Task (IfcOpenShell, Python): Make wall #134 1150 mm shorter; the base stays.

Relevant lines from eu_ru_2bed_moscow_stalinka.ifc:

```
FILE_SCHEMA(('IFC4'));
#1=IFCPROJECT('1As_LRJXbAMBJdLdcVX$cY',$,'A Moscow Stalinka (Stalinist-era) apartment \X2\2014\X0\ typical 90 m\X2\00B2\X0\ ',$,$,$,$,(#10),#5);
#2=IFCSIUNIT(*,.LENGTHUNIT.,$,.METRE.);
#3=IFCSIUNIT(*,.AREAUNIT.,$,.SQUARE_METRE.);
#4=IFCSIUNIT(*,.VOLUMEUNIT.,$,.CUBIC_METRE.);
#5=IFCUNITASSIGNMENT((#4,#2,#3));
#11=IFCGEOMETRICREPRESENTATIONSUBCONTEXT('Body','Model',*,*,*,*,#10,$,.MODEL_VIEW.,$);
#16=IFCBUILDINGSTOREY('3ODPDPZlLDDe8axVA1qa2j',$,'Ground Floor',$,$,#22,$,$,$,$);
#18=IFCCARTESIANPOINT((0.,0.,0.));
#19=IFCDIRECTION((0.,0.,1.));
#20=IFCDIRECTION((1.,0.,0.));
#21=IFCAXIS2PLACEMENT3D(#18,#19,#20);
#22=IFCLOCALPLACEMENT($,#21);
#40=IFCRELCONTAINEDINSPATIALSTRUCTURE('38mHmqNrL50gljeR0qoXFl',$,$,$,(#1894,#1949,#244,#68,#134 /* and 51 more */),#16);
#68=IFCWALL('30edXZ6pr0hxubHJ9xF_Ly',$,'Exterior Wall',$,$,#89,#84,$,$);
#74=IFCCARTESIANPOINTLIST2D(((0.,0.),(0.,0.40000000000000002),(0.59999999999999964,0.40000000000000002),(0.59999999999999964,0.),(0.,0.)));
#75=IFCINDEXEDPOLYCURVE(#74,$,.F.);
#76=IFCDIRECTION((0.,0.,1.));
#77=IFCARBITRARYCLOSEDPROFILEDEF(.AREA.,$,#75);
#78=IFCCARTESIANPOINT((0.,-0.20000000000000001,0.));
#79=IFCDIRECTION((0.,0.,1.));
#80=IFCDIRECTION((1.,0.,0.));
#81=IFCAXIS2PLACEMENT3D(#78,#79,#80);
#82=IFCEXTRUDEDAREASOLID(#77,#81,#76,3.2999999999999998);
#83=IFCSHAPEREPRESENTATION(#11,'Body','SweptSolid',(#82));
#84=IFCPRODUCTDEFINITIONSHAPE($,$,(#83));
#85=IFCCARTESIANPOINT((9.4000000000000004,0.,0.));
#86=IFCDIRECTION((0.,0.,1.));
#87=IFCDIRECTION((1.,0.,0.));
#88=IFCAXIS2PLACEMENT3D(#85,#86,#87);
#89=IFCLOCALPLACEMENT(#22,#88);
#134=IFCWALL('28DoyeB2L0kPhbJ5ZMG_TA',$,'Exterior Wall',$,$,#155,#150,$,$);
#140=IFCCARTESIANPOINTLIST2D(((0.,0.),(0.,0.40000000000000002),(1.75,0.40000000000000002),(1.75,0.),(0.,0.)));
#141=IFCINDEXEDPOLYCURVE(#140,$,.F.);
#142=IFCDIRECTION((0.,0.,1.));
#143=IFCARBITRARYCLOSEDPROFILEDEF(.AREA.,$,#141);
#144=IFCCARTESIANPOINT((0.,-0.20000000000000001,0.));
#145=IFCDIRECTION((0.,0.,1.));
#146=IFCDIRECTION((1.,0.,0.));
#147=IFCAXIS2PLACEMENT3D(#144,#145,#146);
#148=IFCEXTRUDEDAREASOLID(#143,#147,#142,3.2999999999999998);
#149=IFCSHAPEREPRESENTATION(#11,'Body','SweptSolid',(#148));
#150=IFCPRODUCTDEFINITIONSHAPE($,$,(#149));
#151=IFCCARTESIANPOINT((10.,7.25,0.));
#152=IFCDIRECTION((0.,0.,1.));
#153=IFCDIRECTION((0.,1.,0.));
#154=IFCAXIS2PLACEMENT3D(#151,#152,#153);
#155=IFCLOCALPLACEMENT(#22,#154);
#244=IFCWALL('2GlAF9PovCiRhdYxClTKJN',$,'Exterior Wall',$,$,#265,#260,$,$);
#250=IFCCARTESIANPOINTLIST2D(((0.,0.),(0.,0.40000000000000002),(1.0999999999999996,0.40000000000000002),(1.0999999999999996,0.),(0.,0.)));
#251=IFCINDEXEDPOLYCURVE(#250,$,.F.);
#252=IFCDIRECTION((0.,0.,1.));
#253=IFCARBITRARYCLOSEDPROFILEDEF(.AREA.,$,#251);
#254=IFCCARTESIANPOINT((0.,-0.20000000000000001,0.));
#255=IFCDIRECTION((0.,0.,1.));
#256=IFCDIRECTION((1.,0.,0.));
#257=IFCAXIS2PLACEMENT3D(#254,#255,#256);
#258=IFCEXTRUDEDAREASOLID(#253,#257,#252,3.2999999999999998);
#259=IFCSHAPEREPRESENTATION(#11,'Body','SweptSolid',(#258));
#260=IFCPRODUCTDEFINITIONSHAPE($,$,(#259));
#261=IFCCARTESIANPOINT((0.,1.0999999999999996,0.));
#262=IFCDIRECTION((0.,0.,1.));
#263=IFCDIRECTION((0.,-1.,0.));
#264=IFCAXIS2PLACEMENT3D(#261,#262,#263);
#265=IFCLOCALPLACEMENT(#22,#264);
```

```python
import ifcopenshell
import ifcopenshell.geom
import ifcopenshell.util.representation
import ifcopenshell.util.shape
import ifcopenshell.util.unit

model = ifcopenshell.open("eu_ru_2bed_moscow_stalinka.ifc")
unit_scale = ifcopenshell.util.unit.calculate_unit_scale(model)
settings = ifcopenshell.geom.settings()


def volume(element):
    """Net volume in cubic metres, openings subtracted."""
    shape = ifcopenshell.geom.create_shape(settings, element)
    return ifcopenshell.util.shape.get_volume(shape.geometry)


wall = model.by_guid("28DoyeB2L0kPhbJ5ZMG_TA")
before = volume(wall)

body = ifcopenshell.util.representation.get_representation(wall, "Model", "Body")
solid = body.Items[0]
old_height = solid.Depth
solid.Depth -= 1.15 / unit_scale
after = volume(wall)

print(f"height {old_height:g} -> {solid.Depth:g}, volume {before:.3f} -> {after:.3f} m3")

model.write("eu_ru_2bed_moscow_stalinka_rev.ifc")
```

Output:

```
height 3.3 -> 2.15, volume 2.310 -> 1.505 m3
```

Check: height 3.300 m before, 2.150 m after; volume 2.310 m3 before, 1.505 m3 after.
